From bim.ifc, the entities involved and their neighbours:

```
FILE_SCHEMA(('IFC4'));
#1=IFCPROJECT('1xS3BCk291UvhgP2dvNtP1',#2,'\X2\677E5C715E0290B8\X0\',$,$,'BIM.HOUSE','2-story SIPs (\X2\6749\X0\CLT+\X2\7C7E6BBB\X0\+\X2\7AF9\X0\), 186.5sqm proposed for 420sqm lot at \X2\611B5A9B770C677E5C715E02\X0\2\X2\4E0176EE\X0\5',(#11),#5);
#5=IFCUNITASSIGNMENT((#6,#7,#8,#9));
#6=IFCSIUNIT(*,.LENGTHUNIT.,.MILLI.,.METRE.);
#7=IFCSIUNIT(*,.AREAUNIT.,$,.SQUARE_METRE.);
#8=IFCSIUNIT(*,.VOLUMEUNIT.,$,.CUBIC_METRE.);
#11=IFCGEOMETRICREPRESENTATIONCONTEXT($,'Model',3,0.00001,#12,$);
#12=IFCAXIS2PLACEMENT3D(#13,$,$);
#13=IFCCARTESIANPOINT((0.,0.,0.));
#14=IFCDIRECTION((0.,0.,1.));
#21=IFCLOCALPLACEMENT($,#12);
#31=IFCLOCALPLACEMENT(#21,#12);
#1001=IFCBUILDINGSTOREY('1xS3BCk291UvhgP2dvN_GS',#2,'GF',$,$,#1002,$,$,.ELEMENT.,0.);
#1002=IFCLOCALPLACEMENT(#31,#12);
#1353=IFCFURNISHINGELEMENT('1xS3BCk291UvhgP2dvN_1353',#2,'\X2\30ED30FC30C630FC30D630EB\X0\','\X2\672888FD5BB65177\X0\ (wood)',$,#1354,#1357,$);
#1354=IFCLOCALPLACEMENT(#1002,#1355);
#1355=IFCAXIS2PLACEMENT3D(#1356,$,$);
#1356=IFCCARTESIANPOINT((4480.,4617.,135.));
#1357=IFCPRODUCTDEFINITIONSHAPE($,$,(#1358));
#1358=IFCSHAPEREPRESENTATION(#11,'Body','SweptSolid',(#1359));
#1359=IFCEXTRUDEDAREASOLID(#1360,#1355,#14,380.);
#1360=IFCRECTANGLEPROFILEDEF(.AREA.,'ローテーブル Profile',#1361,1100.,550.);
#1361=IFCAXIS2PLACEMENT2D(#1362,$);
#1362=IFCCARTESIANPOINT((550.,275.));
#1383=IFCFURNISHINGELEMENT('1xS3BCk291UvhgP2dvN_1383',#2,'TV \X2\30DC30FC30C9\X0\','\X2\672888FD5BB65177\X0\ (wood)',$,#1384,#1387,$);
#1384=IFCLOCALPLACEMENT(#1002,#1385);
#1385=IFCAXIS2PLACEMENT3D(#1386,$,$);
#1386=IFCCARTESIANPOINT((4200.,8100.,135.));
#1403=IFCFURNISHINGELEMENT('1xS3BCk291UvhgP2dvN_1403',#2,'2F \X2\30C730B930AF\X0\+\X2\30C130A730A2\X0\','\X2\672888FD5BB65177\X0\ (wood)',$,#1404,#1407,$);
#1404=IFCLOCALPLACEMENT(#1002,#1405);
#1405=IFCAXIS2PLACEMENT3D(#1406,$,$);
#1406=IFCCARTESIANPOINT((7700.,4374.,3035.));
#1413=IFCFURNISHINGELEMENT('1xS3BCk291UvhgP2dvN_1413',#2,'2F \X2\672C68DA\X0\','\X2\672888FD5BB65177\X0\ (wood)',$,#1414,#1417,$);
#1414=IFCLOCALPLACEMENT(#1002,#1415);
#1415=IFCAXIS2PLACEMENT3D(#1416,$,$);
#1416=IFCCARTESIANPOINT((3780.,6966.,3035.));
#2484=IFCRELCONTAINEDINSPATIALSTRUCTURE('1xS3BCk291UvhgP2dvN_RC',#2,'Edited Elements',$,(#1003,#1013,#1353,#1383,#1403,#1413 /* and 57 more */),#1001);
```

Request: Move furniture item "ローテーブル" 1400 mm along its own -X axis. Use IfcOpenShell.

```python
import ifcopenshell
import ifcopenshell.api.geometry
import ifcopenshell.util.placement

model = ifcopenshell.open("bim.ifc")

item = model.by_id(1353)
matrix = ifcopenshell.util.placement.get_local_placement(item.ObjectPlacement)
matrix[:3, 3] -= matrix[:3, 0] * 1400.0
ifcopenshell.api.geometry.edit_object_placement(model, product=item, matrix=matrix, is_si=False)

print(ifcopenshell.util.placement.get_local_placement(item.ObjectPlacement).round(3) + 0.0)

model.write("bim-out.ifc")
```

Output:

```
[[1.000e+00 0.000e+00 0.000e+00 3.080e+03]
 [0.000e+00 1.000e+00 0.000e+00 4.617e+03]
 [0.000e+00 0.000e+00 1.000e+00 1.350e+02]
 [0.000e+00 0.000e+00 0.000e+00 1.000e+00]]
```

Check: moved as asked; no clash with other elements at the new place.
